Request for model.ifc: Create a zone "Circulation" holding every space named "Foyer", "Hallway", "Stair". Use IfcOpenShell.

First a look at what the model holds.

```python
import ifcopenshell

model = ifcopenshell.open("model.ifc")
print(model.schema)
seen = {}
for space in model.by_type("IfcSpace"):
    seen[space.LongName] = seen.get(space.LongName, 0) + 1
for name, count in sorted(seen.items(), key=str):
    print(count, "x", name)
print("zones:", [z.Name for z in model.by_type("IfcZone")][:20])
```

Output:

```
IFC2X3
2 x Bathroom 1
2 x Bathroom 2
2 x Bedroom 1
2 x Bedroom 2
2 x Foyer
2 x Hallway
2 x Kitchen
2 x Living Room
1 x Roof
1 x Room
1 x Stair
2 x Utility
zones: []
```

```python
import ifcopenshell
import ifcopenshell.api.group
import ifcopenshell.api.root

model = ifcopenshell.open("model.ifc")

names = {"Foyer", "Hallway", "Stair"}
spaces = [s for s in model.by_type("IfcSpace") if s.LongName in names]

zone = ifcopenshell.api.root.create_entity(model, ifc_class="IfcZone", name="Circulation")
ifcopenshell.api.group.assign_group(model, products=spaces, group=zone)
print(len(spaces), "spaces in", zone.Name)

model.write("model-out.ifc")
```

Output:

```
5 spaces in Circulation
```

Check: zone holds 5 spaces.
